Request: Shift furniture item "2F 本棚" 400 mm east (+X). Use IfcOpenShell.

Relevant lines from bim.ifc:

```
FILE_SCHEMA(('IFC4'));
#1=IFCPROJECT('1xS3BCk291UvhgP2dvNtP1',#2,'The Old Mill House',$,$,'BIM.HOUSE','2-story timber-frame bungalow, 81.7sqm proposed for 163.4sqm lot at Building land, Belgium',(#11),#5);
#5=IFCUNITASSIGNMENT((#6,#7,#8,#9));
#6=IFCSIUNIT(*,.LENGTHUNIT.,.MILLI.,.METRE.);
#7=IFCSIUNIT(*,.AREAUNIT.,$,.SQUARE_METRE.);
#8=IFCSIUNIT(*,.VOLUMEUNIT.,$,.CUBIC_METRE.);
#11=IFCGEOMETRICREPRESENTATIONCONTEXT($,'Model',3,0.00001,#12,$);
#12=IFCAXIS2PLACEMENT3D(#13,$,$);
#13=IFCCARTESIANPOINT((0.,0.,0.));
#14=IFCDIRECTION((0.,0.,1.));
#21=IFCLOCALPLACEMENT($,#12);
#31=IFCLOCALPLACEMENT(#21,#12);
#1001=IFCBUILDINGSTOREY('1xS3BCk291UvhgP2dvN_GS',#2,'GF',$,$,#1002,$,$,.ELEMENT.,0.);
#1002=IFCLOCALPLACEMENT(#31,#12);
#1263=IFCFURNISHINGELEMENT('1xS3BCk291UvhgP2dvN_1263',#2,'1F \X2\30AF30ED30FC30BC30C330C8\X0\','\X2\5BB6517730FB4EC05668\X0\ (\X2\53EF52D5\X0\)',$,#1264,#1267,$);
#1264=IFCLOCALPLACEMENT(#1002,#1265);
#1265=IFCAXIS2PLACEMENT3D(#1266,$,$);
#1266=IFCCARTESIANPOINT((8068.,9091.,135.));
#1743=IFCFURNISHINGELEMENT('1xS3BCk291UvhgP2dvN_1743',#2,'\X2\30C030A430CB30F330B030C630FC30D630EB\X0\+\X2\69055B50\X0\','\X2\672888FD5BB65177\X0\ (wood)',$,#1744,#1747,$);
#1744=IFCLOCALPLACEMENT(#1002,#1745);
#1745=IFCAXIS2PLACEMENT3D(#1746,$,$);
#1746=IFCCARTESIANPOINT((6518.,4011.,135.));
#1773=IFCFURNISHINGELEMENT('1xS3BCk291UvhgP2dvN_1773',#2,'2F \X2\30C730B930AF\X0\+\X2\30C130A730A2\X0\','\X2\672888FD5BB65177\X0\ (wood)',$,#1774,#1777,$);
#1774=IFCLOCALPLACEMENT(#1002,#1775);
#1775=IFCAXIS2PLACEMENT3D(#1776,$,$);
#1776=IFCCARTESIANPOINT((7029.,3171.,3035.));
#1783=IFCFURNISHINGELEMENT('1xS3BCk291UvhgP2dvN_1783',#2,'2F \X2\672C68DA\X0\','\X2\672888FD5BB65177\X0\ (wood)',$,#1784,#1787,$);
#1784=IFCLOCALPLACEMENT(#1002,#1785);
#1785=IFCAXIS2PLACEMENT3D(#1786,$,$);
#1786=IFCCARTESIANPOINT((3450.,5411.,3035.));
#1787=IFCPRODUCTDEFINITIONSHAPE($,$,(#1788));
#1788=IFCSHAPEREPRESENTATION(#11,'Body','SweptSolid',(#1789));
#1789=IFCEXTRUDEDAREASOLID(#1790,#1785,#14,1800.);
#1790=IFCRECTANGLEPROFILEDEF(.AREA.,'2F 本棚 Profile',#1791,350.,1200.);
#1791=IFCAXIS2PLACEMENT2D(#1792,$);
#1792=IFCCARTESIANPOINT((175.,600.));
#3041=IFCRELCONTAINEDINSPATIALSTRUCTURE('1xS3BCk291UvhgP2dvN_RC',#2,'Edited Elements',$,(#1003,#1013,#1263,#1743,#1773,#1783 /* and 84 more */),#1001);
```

```python
import ifcopenshell
import ifcopenshell.api.geometry
import ifcopenshell.util.placement

model = ifcopenshell.open("bim.ifc")

item = model.by_id(1783)
matrix = ifcopenshell.util.placement.get_local_placement(item.ObjectPlacement)
matrix[0, 3] += 400.0
ifcopenshell.api.geometry.edit_object_placement(model, product=item, matrix=matrix, is_si=False)

print(ifcopenshell.util.placement.get_local_placement(item.ObjectPlacement).round(3) + 0.0)

model.write("bim_rev.ifc")
```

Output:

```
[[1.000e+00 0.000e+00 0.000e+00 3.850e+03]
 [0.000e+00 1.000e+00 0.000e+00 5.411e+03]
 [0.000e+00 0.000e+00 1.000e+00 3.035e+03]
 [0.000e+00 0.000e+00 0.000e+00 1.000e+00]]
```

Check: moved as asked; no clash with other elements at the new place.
